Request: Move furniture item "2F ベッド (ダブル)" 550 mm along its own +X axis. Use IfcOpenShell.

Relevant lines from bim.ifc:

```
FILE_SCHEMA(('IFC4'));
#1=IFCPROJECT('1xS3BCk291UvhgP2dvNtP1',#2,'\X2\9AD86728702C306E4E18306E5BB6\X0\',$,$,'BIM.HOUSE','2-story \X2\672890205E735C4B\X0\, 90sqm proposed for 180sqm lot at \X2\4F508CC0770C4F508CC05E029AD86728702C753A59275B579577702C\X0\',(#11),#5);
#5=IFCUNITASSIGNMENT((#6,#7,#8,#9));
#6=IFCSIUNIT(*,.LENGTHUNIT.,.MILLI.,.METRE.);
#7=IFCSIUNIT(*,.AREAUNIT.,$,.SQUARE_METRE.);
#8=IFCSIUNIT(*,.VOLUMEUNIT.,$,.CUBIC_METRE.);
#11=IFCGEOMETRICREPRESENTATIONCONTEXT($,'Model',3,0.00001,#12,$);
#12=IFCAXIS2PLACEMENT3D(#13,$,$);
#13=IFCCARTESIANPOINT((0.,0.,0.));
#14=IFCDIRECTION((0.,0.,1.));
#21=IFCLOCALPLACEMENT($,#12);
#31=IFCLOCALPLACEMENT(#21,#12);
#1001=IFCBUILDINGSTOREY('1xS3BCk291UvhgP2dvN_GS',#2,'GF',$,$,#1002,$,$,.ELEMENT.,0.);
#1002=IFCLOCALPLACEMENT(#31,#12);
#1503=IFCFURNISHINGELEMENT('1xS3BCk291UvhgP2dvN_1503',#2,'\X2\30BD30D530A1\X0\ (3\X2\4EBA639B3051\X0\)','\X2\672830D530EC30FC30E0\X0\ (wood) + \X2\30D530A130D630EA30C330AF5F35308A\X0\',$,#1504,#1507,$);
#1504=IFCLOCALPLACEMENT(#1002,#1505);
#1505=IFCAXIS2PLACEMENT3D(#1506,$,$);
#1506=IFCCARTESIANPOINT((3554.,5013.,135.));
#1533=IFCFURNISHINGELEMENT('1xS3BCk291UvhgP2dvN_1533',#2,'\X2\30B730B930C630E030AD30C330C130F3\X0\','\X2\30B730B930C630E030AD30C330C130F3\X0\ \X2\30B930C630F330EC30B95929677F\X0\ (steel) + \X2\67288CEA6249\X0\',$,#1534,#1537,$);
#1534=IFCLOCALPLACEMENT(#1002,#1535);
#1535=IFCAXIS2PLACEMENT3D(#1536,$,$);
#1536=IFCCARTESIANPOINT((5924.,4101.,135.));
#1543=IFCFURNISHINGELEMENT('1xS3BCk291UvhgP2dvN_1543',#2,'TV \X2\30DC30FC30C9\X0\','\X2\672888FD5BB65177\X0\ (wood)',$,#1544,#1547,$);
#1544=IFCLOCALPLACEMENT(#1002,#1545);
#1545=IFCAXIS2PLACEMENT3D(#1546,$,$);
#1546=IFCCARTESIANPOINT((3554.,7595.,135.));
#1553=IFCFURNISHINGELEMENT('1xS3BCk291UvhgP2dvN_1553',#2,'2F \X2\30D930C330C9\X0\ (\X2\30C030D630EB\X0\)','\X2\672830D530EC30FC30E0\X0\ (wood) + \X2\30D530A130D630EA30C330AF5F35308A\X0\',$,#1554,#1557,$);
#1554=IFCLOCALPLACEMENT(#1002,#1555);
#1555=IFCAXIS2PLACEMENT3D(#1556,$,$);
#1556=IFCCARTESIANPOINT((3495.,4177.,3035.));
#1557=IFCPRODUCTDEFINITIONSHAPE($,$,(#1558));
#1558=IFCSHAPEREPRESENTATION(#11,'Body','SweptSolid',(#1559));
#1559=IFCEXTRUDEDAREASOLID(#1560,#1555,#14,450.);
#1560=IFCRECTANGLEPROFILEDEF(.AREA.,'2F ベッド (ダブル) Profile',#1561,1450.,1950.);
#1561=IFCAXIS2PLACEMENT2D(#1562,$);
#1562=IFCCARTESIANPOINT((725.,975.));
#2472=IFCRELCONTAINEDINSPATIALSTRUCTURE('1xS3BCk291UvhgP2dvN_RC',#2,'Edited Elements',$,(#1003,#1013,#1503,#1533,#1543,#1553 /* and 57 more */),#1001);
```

```python
import ifcopenshell
import ifcopenshell.api.geometry
import ifcopenshell.util.placement
import ifcopenshell.util.unit

model = ifcopenshell.open("bim.ifc")
unit_scale = ifcopenshell.util.unit.calculate_unit_scale(model)

item = model.by_id(1553)
matrix = ifcopenshell.util.placement.get_local_placement(item.ObjectPlacement)
matrix[:3, 3] += matrix[:3, 0] * 0.55 / unit_scale
ifcopenshell.api.geometry.edit_object_placement(model, product=item, matrix=matrix, is_si=False)

print(ifcopenshell.util.placement.get_local_placement(item.ObjectPlacement).round(3) + 0.0)

model.write("bim_updated.ifc")
```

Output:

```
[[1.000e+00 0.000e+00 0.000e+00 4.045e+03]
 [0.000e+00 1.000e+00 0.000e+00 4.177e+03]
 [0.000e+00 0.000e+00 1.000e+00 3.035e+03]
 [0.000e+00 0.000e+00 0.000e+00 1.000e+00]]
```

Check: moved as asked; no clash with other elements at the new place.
